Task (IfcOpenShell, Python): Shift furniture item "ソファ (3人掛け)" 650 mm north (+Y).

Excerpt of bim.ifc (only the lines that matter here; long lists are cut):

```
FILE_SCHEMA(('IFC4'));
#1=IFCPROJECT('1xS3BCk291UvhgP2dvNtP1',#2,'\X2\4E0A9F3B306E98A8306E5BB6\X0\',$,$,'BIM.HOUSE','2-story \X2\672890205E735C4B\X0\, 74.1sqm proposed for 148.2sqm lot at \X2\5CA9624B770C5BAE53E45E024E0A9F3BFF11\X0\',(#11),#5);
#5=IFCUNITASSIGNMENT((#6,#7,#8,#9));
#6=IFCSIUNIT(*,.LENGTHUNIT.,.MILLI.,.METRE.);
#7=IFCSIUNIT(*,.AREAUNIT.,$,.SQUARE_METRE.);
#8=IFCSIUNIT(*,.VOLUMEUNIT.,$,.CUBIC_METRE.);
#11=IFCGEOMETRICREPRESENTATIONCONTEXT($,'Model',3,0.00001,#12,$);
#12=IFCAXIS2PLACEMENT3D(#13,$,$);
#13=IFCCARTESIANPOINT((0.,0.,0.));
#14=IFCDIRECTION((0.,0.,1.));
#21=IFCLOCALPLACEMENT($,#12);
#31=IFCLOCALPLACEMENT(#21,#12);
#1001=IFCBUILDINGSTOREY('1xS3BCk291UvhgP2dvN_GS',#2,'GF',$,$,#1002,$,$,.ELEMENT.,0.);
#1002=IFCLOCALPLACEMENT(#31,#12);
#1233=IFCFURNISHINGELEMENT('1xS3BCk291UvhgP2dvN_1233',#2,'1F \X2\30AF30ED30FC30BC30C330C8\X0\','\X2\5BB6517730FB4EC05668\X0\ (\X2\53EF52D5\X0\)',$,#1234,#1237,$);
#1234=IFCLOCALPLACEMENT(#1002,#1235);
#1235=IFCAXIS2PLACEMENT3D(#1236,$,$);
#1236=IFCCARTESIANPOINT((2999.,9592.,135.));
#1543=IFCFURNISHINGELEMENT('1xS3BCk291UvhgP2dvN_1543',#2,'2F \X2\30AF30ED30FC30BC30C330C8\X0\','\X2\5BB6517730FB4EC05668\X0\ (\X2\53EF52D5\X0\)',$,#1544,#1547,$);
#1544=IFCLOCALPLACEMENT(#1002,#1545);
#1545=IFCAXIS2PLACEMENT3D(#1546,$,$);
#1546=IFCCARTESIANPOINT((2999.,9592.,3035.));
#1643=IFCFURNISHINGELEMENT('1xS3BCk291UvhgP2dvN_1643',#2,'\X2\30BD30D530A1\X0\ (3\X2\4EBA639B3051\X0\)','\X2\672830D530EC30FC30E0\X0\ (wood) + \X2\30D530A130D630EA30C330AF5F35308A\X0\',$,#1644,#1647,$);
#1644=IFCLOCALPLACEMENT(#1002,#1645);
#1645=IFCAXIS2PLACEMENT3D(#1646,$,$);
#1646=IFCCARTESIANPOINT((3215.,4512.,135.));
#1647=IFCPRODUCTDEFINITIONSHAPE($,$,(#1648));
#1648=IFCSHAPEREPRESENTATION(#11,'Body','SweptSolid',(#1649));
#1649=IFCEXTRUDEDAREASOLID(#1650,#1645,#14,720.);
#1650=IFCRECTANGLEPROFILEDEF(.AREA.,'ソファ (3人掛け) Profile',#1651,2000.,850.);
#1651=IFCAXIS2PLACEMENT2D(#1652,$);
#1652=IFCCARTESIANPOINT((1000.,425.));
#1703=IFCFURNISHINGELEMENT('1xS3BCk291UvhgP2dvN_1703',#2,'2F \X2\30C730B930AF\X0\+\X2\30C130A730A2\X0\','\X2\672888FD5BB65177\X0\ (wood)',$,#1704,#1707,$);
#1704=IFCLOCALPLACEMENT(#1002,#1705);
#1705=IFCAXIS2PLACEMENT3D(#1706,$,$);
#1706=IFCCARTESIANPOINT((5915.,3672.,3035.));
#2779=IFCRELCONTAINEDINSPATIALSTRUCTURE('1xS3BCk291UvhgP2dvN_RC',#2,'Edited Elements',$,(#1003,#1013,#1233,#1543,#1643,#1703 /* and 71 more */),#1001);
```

```python
import ifcopenshell
import ifcopenshell.api.geometry
import ifcopenshell.util.placement

model = ifcopenshell.open("bim.ifc")

item = model.by_guid("1xS3BCk291UvhgP2dvN_1643")
matrix = ifcopenshell.util.placement.get_local_placement(item.ObjectPlacement)
matrix[1, 3] += 650.0
ifcopenshell.api.geometry.edit_object_placement(model, product=item, matrix=matrix, is_si=False)

print(ifcopenshell.util.placement.get_local_placement(item.ObjectPlacement).round(3) + 0.0)

model.write("bim_edited.ifc")
```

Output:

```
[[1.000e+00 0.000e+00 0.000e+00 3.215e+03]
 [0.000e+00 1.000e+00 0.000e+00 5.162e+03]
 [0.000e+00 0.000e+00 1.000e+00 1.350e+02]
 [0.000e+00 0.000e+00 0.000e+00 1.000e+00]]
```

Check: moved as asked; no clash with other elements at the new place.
